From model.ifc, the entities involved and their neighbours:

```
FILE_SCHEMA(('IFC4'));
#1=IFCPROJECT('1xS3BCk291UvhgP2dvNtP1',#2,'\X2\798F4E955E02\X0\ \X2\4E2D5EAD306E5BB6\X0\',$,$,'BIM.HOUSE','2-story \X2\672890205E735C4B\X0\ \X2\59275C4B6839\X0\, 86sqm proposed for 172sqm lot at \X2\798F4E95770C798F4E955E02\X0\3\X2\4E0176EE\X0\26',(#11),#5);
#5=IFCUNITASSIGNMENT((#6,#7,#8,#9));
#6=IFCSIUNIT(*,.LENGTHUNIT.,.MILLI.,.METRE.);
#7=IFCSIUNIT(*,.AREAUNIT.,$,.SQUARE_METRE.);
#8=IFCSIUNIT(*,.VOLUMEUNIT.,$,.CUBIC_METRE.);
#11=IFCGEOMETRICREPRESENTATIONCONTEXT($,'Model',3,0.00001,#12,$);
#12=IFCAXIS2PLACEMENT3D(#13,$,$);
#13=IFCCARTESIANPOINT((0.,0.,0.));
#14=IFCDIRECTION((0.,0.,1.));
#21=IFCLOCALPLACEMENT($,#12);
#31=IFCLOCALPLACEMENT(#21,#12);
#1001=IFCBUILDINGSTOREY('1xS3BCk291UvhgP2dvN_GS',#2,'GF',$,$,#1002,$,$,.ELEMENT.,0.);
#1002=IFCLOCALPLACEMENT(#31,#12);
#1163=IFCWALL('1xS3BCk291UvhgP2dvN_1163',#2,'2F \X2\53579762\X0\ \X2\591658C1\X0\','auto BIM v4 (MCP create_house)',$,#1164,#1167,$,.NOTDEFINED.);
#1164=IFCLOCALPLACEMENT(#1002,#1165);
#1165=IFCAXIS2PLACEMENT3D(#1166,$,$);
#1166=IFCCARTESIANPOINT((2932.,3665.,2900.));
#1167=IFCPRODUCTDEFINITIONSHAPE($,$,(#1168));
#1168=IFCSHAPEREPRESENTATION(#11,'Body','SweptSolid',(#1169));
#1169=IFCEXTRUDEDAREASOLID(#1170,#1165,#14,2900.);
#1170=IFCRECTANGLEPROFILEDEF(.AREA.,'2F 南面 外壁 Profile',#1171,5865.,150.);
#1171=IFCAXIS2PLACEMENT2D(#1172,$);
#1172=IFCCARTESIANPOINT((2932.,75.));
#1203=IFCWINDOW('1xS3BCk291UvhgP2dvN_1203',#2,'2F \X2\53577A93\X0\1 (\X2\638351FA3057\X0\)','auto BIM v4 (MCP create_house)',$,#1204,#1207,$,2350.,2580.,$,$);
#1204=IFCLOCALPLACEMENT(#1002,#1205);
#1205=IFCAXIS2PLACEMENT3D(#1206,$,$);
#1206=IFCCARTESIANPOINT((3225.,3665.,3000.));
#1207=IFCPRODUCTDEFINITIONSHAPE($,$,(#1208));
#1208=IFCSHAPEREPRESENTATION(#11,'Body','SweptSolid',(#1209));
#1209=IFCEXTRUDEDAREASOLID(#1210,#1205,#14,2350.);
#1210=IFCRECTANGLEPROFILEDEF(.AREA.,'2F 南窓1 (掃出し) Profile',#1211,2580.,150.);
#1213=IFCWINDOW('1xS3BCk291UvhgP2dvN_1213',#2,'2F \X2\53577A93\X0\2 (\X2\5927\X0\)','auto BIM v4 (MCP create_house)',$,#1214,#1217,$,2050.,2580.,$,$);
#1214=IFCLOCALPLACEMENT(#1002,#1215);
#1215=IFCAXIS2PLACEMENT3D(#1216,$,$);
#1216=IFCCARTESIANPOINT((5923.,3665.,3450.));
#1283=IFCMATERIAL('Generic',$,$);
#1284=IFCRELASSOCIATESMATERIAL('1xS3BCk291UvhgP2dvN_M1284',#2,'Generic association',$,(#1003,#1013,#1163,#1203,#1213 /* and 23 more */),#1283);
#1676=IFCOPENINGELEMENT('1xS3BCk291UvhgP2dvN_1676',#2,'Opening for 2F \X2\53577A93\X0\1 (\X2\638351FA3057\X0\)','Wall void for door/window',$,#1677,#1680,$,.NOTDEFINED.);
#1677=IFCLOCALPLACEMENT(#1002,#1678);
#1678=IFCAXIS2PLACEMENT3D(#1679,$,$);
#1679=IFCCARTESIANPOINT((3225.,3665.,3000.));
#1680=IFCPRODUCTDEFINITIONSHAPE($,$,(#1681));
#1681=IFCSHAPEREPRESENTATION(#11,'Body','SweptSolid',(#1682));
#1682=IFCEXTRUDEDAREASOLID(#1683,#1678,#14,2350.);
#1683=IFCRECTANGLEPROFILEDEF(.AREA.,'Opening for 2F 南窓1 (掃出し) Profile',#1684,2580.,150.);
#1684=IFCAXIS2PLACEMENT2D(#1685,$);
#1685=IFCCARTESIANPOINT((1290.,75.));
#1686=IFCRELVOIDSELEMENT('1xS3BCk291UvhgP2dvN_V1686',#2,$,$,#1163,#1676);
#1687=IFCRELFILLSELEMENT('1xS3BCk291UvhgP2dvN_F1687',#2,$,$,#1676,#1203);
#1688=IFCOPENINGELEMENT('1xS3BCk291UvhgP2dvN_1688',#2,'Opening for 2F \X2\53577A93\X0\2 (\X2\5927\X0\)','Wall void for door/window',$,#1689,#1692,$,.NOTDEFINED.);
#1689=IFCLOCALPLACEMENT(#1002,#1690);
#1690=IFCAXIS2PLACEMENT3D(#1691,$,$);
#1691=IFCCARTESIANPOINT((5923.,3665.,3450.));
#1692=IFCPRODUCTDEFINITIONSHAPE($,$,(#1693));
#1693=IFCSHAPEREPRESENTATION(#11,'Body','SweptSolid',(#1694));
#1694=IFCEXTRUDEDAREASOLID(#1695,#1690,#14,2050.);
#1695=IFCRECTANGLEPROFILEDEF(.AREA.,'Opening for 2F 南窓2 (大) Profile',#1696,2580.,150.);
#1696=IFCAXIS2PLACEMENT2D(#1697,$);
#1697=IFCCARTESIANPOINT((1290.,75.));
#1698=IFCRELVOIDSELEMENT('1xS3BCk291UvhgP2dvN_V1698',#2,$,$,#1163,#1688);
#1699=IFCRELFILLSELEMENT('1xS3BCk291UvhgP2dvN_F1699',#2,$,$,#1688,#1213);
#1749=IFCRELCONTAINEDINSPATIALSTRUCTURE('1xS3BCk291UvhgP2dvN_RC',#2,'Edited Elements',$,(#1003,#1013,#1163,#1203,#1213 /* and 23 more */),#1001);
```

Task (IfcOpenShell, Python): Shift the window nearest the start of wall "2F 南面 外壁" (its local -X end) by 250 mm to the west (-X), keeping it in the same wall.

```python
import ifcopenshell
import ifcopenshell.api.geometry
import ifcopenshell.util.placement
import ifcopenshell.util.unit

model = ifcopenshell.open("model.ifc")
unit_scale = ifcopenshell.util.unit.calculate_unit_scale(model)

window = model.by_guid("1xS3BCk291UvhgP2dvN_1203")
opening = window.FillsVoids[0].RelatingOpeningElement
wall = opening.VoidsElements[0].RelatingBuildingElement

wall_matrix = ifcopenshell.util.placement.get_local_placement(wall.ObjectPlacement)
shift = wall_matrix[:3, 0] * -0.25 / unit_scale
before = ifcopenshell.util.placement.get_local_placement(window.ObjectPlacement)[:3, 3].copy()

# The window is not placed relative to its opening, so move both.
for product in (opening, window):
    matrix = ifcopenshell.util.placement.get_local_placement(product.ObjectPlacement)
    matrix[:3, 3] += shift
    ifcopenshell.api.geometry.edit_object_placement(model, product=product, matrix=matrix, is_si=False)

after = ifcopenshell.util.placement.get_local_placement(window.ObjectPlacement)[:3, 3]
print("window moved by", (after - before).round(3) + 0.0)

model.write("model_v2.ifc")
```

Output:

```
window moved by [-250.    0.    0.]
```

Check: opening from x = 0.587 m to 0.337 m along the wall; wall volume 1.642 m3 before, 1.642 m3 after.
